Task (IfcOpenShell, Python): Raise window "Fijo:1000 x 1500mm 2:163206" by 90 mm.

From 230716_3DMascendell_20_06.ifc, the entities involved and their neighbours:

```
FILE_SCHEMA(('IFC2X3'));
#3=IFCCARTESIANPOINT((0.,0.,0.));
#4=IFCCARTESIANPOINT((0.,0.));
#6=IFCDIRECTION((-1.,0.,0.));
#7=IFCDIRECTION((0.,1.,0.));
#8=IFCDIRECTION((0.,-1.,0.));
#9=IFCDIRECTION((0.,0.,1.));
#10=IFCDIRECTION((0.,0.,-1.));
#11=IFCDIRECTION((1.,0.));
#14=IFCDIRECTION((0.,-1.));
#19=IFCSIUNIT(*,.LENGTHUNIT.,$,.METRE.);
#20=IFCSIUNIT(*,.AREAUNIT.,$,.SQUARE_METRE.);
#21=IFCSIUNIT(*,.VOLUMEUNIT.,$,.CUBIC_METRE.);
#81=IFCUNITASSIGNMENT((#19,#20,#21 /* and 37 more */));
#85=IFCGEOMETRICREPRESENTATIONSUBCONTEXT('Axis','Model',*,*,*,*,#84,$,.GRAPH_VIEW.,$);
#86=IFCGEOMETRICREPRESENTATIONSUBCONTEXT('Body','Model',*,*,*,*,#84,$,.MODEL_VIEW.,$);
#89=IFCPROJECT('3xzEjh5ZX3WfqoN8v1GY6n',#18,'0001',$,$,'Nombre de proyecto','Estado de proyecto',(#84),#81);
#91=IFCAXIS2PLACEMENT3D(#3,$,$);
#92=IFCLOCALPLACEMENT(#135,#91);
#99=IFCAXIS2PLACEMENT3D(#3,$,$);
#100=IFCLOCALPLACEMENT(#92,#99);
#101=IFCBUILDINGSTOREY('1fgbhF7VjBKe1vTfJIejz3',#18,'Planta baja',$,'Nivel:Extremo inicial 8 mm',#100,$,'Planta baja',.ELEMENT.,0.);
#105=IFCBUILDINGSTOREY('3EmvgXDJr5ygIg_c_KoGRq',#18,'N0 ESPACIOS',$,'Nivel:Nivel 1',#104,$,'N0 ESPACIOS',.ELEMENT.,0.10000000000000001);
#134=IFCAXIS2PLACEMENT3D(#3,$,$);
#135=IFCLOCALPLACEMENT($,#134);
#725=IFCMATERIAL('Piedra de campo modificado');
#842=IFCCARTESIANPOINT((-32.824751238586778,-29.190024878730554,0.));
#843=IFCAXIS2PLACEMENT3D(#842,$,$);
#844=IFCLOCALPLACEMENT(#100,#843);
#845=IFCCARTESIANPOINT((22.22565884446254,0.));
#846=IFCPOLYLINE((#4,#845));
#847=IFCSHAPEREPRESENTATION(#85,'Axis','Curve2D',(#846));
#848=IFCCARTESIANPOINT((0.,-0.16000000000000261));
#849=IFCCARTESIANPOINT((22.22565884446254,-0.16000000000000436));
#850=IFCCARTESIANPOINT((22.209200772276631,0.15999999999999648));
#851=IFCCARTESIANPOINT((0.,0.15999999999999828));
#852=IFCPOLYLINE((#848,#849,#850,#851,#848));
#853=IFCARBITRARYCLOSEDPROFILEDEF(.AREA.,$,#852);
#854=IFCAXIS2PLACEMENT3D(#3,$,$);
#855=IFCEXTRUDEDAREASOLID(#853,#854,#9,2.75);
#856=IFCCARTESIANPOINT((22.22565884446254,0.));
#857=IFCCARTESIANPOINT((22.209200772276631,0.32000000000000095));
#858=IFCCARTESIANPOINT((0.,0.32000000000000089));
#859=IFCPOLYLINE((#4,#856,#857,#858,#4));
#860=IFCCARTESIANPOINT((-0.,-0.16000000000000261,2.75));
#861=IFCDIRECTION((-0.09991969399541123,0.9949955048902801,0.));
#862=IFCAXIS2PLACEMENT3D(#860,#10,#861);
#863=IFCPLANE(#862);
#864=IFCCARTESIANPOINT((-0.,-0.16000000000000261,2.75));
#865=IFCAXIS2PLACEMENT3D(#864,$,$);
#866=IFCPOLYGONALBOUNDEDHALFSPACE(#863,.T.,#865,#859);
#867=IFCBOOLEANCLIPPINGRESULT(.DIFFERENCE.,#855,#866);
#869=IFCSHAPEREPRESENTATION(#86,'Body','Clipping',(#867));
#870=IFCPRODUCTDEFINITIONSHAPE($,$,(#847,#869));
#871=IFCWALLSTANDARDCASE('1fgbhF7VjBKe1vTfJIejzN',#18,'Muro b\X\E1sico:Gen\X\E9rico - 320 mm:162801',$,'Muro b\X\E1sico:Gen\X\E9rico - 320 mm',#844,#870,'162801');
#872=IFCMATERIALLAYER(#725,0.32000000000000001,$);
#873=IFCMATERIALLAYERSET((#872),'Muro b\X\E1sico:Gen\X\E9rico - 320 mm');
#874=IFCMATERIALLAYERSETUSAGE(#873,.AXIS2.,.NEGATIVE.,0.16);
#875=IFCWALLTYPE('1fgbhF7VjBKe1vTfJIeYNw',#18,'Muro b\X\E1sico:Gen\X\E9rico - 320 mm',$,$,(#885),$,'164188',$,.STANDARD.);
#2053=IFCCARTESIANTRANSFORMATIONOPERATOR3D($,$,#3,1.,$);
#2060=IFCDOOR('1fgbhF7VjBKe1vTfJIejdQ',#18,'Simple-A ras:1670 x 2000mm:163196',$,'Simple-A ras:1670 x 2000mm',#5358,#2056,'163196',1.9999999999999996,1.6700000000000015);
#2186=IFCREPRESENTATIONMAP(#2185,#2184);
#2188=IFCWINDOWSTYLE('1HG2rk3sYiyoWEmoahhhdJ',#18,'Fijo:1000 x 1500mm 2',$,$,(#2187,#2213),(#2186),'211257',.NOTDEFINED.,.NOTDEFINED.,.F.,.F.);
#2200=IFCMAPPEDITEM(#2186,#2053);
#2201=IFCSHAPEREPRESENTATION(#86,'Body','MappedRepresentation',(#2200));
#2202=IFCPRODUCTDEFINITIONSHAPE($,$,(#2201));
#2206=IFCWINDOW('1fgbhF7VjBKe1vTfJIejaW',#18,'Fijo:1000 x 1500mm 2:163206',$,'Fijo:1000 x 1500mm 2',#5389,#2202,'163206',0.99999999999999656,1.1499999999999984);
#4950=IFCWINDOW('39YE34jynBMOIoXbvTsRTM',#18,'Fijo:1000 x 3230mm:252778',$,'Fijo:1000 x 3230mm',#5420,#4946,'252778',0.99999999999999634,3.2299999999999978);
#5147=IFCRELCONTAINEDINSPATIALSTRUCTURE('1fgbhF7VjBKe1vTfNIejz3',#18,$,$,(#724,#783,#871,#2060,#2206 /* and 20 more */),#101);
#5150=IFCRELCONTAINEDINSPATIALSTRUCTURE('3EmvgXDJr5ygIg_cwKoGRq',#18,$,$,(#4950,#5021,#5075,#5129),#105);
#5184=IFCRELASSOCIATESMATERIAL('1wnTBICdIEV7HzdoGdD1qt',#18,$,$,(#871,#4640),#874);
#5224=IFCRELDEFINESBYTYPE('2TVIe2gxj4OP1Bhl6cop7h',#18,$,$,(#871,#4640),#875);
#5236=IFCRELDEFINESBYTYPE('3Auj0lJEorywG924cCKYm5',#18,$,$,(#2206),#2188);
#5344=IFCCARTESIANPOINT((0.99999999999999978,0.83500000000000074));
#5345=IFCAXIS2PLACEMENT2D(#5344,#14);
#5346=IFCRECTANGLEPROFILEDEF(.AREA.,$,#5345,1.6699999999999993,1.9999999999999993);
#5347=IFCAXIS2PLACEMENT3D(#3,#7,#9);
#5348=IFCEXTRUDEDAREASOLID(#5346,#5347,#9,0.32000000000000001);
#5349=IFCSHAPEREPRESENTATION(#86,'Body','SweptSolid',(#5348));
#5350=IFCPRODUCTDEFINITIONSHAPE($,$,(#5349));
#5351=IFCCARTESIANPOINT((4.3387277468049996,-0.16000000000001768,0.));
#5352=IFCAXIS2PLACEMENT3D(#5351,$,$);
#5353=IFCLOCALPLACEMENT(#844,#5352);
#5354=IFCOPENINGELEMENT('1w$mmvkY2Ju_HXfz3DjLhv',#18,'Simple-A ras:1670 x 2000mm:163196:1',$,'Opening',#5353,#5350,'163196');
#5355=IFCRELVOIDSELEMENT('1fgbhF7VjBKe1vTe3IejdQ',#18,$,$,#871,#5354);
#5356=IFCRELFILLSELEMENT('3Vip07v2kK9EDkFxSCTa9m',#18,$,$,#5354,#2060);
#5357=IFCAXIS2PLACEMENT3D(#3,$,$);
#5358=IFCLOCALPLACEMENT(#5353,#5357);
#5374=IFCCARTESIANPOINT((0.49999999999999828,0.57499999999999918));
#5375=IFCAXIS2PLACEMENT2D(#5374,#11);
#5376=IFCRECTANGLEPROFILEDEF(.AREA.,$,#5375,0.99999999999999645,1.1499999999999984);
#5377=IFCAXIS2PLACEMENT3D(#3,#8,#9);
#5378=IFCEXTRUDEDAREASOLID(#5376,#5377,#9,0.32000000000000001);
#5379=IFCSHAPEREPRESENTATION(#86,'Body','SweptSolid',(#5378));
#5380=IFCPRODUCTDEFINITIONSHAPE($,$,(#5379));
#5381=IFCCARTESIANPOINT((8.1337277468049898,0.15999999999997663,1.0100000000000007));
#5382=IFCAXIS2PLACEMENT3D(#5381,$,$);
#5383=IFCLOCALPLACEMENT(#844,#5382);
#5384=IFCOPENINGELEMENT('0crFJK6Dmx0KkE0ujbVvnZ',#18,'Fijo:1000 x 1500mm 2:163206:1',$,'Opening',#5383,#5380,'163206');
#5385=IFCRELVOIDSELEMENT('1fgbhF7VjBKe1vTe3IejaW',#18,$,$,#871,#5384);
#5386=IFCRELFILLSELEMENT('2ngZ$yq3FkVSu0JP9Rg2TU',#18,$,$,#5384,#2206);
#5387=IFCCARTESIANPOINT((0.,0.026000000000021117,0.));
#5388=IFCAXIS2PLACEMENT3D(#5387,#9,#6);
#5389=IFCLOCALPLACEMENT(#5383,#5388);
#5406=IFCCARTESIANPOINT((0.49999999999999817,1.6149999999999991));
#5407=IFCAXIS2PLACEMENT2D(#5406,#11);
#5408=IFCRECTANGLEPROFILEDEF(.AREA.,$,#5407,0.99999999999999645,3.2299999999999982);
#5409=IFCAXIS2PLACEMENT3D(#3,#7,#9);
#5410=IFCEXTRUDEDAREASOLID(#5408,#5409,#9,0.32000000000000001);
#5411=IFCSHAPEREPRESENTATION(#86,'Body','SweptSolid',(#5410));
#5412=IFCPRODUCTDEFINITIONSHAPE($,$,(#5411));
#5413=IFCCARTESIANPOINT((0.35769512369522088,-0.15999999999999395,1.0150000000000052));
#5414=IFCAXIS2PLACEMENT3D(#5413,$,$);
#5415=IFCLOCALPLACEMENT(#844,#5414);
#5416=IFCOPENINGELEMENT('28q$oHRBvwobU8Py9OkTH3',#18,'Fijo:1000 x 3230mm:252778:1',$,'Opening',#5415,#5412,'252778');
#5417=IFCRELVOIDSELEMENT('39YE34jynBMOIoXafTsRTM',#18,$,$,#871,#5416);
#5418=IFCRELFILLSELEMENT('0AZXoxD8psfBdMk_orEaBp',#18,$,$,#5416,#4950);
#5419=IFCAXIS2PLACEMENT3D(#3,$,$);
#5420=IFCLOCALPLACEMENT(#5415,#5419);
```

```python
import numpy as np
import ifcopenshell
import ifcopenshell.api.geometry
import ifcopenshell.util.placement
import ifcopenshell.util.unit

model = ifcopenshell.open("230716_3DMascendell_20_06.ifc")
unit_scale = ifcopenshell.util.unit.calculate_unit_scale(model)

window = model.by_guid("1fgbhF7VjBKe1vTfJIejaW")
opening = window.FillsVoids[0].RelatingOpeningElement
dz = 0.09

shift = np.array([0.0, 0.0, dz])
# The window is placed relative to its opening, so it follows when the opening moves.
matrix = ifcopenshell.util.placement.get_local_placement(opening.ObjectPlacement)
matrix[:3, 3] += shift
ifcopenshell.api.geometry.edit_object_placement(
    model, product=opening, matrix=matrix, is_si=False, should_transform_children=True
)

print(f"moved by {dz * unit_scale:+.3f} m")

model.write("230716_3DMascendell_20_06_updated.ifc")
```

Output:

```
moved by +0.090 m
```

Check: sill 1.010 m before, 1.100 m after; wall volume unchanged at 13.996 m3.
